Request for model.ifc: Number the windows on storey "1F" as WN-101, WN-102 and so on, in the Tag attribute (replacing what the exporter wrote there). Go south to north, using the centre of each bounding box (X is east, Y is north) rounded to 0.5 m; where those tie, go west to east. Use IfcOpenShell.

First a look at what the model holds.

```python
import ifcopenshell
import ifcopenshell.util.element
import ifcopenshell.util.placement

model = ifcopenshell.open("model.ifc")
print(model.schema)
storey = next(s for s in model.by_type("IfcBuildingStorey") if s.Name == "1F")
windows = [e for e in ifcopenshell.util.element.get_decomposition(storey) if e.is_a("IfcWindow")]
for e in sorted(windows, key=lambda e: e.id()):
    origin = ifcopenshell.util.placement.get_local_placement(e.ObjectPlacement)[:3, 3]
    print(e.id(), e.Tag, e.Name, origin.round(2) + 0.0, sep=" | ")
```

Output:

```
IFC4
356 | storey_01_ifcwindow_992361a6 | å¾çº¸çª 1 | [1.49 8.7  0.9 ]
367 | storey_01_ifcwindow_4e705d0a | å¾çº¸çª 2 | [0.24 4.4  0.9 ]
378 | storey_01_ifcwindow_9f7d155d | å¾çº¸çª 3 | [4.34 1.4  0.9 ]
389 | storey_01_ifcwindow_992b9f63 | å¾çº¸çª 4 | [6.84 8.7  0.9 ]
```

```python
import ifcopenshell
import ifcopenshell.geom
import ifcopenshell.util.element
import ifcopenshell.util.shape

model = ifcopenshell.open("model.ifc")
settings = ifcopenshell.geom.settings()
settings.set("use-world-coords", True)


def centre(element):
    shape = ifcopenshell.geom.create_shape(settings, element)
    return ifcopenshell.util.shape.get_bbox_centroid(shape.geometry)


storey = next(s for s in model.by_type("IfcBuildingStorey") if s.Name == "1F")
windows = [e for e in ifcopenshell.util.element.get_decomposition(storey) if e.is_a("IfcWindow")]

# Insertion points can sit at a corner or the storey origin, so sort by the geometry (in metres).
centres = {e: centre(e) for e in windows}
windows.sort(key=lambda e: (round(centres[e][1] / 0.5), centres[e][0]))

for i, e in enumerate(windows, start=1):
    number = f"WN-1{i:02d}"
    e.Tag = number
    print(e.id(), number)

model.write("model-out.ifc")
```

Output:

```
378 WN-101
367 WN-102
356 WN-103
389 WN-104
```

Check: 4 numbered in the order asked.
